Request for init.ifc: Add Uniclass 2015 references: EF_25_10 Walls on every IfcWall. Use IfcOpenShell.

First a look at what the model holds.

```python
import ifcopenshell

model = ifcopenshell.open("init.ifc")
print(model.schema)
print("classifications:", [c.Name for c in model.by_type("IfcClassification")])
for ifc_class in ("IfcDoor", "IfcRoof", "IfcStair", "IfcWall", "IfcWindow"):
    print(ifc_class, len(model.by_type(ifc_class)))
```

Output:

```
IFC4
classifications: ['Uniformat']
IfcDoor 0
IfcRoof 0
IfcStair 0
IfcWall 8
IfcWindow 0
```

```python
import ifcopenshell
import ifcopenshell.api.classification

model = ifcopenshell.open("init.ifc")

system = ifcopenshell.api.classification.add_classification(model, classification="Uniclass 2015")

codes = {
    "IfcWall": ("EF_25_10", "Walls"),
}
for ifc_class, (code, name) in codes.items():
    products = model.by_type(ifc_class)
    ifcopenshell.api.classification.add_reference(
        model, products=products, classification=system, identification=code, name=name
    )
    print(code, len(products))

model.write("init_updated.ifc")
```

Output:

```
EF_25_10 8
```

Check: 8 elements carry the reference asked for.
